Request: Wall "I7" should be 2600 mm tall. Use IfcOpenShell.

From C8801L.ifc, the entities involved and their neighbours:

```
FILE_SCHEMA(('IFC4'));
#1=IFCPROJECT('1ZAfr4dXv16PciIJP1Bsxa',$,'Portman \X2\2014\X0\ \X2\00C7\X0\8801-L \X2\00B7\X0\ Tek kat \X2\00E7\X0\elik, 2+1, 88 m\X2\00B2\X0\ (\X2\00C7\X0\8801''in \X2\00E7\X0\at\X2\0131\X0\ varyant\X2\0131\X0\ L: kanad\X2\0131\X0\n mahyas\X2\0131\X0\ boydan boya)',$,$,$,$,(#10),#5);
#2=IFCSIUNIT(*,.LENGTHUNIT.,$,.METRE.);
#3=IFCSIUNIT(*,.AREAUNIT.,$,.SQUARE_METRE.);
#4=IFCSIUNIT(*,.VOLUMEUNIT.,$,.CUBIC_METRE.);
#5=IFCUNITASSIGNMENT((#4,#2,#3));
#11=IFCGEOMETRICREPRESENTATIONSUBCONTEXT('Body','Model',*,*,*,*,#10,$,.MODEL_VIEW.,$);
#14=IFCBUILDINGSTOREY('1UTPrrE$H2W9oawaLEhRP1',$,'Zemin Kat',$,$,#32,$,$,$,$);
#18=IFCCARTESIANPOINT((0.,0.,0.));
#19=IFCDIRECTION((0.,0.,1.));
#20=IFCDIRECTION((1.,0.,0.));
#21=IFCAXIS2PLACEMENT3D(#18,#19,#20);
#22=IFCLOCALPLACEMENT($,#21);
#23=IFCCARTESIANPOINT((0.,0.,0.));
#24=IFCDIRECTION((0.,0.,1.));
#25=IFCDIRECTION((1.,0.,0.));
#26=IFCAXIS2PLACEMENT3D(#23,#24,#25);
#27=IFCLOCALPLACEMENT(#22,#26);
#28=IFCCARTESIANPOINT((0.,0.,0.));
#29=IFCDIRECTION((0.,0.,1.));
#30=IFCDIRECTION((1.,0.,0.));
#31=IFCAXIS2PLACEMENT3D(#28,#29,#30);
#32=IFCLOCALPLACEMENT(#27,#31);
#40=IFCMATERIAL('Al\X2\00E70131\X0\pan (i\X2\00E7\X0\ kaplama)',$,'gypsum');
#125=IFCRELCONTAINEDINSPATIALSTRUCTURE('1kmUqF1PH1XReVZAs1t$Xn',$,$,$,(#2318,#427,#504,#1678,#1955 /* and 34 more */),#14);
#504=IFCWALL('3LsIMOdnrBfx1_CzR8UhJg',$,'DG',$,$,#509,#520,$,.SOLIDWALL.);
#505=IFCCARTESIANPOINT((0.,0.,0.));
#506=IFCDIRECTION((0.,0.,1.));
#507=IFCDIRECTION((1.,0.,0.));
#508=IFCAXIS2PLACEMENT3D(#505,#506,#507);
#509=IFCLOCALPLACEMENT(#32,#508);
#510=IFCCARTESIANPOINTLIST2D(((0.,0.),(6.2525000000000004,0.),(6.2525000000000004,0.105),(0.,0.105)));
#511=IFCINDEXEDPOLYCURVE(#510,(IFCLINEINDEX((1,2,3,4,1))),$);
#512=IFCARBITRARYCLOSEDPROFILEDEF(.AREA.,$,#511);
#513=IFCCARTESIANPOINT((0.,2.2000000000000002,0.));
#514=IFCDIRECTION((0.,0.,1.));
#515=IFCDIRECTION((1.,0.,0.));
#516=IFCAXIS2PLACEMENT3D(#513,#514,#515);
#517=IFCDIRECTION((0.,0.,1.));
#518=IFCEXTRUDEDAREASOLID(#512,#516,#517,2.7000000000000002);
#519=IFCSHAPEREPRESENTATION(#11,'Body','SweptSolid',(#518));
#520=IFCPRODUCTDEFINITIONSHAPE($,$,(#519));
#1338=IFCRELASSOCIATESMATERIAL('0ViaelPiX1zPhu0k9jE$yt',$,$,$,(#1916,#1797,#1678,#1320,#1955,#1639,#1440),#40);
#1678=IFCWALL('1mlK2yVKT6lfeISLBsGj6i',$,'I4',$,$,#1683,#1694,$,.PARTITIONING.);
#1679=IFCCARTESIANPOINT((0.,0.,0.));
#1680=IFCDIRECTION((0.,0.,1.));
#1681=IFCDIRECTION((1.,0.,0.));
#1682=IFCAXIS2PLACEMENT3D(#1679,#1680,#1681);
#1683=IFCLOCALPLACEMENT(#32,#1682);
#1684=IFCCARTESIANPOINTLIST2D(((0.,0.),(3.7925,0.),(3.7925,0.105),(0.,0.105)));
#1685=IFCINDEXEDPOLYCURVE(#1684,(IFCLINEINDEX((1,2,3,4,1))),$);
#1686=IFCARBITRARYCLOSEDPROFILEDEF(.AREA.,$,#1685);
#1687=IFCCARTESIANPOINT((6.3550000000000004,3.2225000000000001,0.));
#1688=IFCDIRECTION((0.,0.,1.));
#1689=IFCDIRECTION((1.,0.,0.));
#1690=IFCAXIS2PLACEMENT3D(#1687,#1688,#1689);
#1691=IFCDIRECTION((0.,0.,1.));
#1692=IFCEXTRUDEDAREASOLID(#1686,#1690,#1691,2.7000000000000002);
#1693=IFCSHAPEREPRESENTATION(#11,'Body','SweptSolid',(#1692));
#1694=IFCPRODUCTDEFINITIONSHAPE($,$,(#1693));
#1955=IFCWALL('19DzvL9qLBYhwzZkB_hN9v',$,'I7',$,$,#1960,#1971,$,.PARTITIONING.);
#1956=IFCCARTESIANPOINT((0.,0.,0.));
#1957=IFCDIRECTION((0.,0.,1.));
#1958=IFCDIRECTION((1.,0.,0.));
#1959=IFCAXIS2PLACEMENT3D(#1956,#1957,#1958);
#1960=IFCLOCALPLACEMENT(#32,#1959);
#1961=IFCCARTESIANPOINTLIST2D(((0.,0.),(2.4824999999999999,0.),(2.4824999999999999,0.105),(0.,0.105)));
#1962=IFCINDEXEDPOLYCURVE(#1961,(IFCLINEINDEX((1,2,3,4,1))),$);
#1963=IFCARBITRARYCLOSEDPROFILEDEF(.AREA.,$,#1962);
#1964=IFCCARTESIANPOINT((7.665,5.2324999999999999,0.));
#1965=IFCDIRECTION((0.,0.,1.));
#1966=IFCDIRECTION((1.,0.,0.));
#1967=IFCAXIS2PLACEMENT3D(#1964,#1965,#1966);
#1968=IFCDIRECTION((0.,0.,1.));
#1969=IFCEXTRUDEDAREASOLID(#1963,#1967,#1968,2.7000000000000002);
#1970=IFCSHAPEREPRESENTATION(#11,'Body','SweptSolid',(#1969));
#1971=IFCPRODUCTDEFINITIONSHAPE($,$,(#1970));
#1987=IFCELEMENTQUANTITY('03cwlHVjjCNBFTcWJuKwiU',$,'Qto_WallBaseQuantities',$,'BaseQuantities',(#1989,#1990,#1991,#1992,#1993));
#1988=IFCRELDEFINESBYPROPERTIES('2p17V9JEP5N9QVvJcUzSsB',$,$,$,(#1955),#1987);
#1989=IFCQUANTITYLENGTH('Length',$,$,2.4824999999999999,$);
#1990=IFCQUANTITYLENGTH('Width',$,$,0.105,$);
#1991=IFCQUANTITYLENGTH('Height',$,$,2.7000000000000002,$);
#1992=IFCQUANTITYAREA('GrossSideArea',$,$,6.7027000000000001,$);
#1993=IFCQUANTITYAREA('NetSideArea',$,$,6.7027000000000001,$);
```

```python
import ifcopenshell
import ifcopenshell.api.pset
import ifcopenshell.geom
import ifcopenshell.util.element
import ifcopenshell.util.representation
import ifcopenshell.util.shape
import ifcopenshell.util.unit

model = ifcopenshell.open("C8801L.ifc")
unit_scale = ifcopenshell.util.unit.calculate_unit_scale(model)
area_scale = ifcopenshell.util.unit.calculate_unit_scale(model, "AREAUNIT")
settings = ifcopenshell.geom.settings()


def volume(element):
    """Net volume in cubic metres, openings subtracted."""
    shape = ifcopenshell.geom.create_shape(settings, element)
    return ifcopenshell.util.shape.get_volume(shape.geometry)


wall = model.by_guid("19DzvL9qLBYhwzZkB_hN9v")
before = volume(wall)

body = ifcopenshell.util.representation.get_representation(wall, "Model", "Body")
solid = body.Items[0]
old_height = solid.Depth
solid.Depth = 2.6
after = volume(wall)
thickness = 0.105  # wall thickness in metres

# Update the stored height, areas and volumes.
qto = model.by_id(ifcopenshell.util.element.get_pset(wall, "Qto_WallBaseQuantities", should_inherit=False)["id"])
ifcopenshell.api.pset.edit_qto(model, qto=qto, properties={
    "Height": solid.Depth,
    "GrossSideArea": ifcopenshell.util.element.get_pset(wall, "Qto_WallBaseQuantities", "GrossSideArea") * solid.Depth / old_height,
    "NetSideArea": after / thickness / area_scale,
})

print(f"height {old_height:g} -> {solid.Depth:g}, volume {before:.3f} -> {after:.3f} m3")

model.write("C8801L_updated.ifc")
```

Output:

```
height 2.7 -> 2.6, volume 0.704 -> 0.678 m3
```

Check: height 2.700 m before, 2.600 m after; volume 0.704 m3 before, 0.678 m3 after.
